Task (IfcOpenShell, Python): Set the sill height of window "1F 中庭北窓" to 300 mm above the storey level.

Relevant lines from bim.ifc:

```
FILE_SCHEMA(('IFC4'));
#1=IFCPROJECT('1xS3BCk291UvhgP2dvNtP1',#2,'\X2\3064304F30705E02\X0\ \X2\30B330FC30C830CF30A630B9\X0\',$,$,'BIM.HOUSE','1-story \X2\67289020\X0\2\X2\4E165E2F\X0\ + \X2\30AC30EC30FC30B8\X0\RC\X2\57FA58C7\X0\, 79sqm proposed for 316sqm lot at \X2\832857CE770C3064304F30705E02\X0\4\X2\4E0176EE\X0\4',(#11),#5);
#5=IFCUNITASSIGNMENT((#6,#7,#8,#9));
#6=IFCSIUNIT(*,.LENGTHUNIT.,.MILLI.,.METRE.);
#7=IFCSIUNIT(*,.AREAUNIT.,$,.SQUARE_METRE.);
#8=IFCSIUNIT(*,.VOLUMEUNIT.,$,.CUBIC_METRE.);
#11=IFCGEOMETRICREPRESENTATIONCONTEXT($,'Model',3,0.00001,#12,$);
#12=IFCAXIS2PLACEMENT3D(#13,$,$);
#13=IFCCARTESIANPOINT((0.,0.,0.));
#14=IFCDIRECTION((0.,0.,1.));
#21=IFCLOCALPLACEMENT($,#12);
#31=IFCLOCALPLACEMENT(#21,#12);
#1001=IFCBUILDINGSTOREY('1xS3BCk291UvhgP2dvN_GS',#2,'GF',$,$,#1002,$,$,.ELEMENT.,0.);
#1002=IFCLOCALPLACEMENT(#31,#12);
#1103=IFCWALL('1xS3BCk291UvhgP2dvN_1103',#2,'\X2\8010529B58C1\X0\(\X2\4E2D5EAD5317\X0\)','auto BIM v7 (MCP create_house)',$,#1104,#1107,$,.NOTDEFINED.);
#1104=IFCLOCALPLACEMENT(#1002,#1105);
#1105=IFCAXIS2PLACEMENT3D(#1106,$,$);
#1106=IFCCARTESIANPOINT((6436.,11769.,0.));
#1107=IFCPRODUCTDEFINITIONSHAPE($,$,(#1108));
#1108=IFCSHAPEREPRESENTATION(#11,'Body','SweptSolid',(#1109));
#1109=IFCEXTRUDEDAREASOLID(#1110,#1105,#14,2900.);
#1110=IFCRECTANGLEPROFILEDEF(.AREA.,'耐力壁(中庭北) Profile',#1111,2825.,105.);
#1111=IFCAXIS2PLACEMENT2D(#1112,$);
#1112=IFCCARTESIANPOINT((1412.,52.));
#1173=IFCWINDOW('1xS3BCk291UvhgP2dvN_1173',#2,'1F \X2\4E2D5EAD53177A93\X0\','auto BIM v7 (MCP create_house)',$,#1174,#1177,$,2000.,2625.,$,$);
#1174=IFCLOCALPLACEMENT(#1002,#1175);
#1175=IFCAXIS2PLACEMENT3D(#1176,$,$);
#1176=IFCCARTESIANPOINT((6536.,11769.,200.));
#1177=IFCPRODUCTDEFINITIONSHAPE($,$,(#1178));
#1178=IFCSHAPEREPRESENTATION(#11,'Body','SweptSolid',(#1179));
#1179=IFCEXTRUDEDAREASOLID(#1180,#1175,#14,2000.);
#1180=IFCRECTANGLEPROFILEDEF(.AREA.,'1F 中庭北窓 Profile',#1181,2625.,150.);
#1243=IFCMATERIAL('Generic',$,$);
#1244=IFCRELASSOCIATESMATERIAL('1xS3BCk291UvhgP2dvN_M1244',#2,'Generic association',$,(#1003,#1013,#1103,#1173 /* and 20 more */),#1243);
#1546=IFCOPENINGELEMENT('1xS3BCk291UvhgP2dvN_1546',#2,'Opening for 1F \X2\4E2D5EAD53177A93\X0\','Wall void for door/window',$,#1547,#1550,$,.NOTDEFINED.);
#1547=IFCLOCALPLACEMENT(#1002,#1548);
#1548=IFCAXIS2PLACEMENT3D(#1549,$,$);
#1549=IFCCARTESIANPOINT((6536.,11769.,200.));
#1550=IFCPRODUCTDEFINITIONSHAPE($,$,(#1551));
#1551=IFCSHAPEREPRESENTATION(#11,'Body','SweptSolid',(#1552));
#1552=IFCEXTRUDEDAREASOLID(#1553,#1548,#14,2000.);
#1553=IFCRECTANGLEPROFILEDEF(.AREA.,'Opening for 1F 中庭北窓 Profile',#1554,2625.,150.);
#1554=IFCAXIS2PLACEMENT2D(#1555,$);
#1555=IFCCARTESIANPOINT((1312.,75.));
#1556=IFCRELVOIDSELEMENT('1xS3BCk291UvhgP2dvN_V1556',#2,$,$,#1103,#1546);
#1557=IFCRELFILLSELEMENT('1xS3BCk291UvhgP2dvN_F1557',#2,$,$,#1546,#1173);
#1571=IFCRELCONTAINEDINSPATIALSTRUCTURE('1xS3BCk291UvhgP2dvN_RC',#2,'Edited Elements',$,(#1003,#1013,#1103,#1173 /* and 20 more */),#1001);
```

```python
import numpy as np
import ifcopenshell
import ifcopenshell.api.geometry
import ifcopenshell.geom
import ifcopenshell.util.element
import ifcopenshell.util.placement
import ifcopenshell.util.shape
import ifcopenshell.util.unit

model = ifcopenshell.open("bim.ifc")
unit_scale = ifcopenshell.util.unit.calculate_unit_scale(model)

window = model.by_id(1173)
opening = window.FillsVoids[0].RelatingOpeningElement
storey = ifcopenshell.util.element.get_container(window, ifc_class="IfcBuildingStorey")
level = ifcopenshell.util.placement.get_local_placement(storey.ObjectPlacement)[2, 3]

# The opening's origin need not be at the sill, so measure its lowest point.
shape = ifcopenshell.geom.create_shape(ifcopenshell.geom.settings(), opening)
bottom = ifcopenshell.util.shape.get_shape_bottom_elevation(shape, shape.geometry) / unit_scale
dz = level + 0.3 / unit_scale - bottom

shift = np.array([0.0, 0.0, dz])
# The window is not placed relative to its opening, so move both.
for product in (opening, window):
    matrix = ifcopenshell.util.placement.get_local_placement(product.ObjectPlacement)
    matrix[:3, 3] += shift
    ifcopenshell.api.geometry.edit_object_placement(model, product=product, matrix=matrix, is_si=False)

print(f"moved by {dz * unit_scale:+.3f} m")

model.write("bim_rev.ifc")
```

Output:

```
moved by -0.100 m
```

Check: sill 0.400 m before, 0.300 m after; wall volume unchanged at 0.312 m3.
